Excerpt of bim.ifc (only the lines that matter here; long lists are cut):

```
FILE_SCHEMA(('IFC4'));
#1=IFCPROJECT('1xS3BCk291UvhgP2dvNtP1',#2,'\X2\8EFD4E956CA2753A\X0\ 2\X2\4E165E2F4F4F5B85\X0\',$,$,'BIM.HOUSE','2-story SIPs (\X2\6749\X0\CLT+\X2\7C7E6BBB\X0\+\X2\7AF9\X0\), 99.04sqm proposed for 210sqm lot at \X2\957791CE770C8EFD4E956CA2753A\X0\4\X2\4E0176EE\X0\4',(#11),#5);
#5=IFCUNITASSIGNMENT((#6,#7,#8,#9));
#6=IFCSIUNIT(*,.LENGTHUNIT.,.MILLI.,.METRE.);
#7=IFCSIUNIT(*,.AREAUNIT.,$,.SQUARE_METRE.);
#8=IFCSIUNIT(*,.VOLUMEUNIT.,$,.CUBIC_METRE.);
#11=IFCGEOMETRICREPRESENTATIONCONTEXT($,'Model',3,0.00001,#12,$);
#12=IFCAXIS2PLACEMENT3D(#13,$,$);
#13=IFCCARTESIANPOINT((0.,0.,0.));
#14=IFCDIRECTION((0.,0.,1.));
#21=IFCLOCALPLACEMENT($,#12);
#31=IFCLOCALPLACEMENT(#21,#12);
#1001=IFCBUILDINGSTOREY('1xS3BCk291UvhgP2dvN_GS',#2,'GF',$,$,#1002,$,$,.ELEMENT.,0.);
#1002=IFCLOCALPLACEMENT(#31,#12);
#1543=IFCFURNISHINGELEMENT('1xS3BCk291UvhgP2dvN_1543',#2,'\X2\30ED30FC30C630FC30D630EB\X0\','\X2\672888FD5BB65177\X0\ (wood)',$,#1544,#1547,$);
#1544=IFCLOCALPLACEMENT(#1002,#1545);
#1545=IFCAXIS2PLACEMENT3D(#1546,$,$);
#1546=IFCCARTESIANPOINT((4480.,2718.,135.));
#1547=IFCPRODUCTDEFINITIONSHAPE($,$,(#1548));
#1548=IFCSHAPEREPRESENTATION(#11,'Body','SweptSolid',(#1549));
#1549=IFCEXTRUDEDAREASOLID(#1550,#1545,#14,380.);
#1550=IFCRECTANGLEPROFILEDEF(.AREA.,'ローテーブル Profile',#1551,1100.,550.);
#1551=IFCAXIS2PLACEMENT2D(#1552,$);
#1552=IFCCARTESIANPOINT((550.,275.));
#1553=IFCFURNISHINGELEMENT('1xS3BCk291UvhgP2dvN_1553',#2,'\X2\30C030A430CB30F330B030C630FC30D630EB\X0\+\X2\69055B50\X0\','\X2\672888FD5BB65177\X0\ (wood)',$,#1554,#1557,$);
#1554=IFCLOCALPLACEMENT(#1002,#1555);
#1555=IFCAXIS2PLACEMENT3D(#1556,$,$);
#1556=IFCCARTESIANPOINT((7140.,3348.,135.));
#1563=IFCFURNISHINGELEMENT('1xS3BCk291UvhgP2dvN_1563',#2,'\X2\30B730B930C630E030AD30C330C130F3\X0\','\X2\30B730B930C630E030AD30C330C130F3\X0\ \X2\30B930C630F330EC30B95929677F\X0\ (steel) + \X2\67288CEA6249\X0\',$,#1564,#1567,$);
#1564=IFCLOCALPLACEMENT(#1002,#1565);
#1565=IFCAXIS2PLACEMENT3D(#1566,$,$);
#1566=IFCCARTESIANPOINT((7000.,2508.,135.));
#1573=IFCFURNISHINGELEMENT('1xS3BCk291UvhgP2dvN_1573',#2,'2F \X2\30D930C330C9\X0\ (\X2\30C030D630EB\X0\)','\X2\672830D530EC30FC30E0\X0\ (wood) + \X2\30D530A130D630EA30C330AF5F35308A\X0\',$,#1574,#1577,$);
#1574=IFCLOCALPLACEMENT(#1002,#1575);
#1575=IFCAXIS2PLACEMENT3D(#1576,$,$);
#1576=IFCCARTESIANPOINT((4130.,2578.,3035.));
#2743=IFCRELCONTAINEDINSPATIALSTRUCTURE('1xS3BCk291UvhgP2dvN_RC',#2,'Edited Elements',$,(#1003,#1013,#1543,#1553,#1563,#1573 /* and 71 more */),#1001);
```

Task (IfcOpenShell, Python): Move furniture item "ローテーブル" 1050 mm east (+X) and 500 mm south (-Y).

```python
import ifcopenshell
import ifcopenshell.api.geometry
import ifcopenshell.util.placement

model = ifcopenshell.open("bim.ifc")

item = model.by_guid("1xS3BCk291UvhgP2dvN_1543")
matrix = ifcopenshell.util.placement.get_local_placement(item.ObjectPlacement)
matrix[0, 3] += 1050.0
matrix[1, 3] -= 500.0
ifcopenshell.api.geometry.edit_object_placement(model, product=item, matrix=matrix, is_si=False)

print(ifcopenshell.util.placement.get_local_placement(item.ObjectPlacement).round(3) + 0.0)

model.write("bim-out.ifc")
```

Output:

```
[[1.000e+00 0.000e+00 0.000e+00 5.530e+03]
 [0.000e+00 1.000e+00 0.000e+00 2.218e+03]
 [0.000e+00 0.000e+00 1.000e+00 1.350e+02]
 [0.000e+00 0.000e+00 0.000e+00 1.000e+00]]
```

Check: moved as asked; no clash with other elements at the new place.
